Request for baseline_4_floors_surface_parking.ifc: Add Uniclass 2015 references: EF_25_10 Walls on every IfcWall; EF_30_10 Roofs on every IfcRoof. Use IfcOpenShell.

First a look at what the model holds.

```python
import ifcopenshell

model = ifcopenshell.open("baseline_4_floors_surface_parking.ifc")
print(model.schema)
print("classifications:", [c.Name for c in model.by_type("IfcClassification")])
for ifc_class in ("IfcDoor", "IfcRoof", "IfcStair", "IfcWall", "IfcWindow"):
    print(ifc_class, len(model.by_type(ifc_class)))
```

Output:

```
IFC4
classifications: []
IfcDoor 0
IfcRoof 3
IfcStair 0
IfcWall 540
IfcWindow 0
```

```python
import ifcopenshell
import ifcopenshell.api.classification

model = ifcopenshell.open("baseline_4_floors_surface_parking.ifc")

system = ifcopenshell.api.classification.add_classification(model, classification="Uniclass 2015")

codes = {
    "IfcWall": ("EF_25_10", "Walls"),
    "IfcRoof": ("EF_30_10", "Roofs"),
}
for ifc_class, (code, name) in codes.items():
    products = model.by_type(ifc_class)
    ifcopenshell.api.classification.add_reference(
        model, products=products, classification=system, identification=code, name=name
    )
    print(code, len(products))

model.write("baseline_4_floors_surface_parking_updated.ifc")
```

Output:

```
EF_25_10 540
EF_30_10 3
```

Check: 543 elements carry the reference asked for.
